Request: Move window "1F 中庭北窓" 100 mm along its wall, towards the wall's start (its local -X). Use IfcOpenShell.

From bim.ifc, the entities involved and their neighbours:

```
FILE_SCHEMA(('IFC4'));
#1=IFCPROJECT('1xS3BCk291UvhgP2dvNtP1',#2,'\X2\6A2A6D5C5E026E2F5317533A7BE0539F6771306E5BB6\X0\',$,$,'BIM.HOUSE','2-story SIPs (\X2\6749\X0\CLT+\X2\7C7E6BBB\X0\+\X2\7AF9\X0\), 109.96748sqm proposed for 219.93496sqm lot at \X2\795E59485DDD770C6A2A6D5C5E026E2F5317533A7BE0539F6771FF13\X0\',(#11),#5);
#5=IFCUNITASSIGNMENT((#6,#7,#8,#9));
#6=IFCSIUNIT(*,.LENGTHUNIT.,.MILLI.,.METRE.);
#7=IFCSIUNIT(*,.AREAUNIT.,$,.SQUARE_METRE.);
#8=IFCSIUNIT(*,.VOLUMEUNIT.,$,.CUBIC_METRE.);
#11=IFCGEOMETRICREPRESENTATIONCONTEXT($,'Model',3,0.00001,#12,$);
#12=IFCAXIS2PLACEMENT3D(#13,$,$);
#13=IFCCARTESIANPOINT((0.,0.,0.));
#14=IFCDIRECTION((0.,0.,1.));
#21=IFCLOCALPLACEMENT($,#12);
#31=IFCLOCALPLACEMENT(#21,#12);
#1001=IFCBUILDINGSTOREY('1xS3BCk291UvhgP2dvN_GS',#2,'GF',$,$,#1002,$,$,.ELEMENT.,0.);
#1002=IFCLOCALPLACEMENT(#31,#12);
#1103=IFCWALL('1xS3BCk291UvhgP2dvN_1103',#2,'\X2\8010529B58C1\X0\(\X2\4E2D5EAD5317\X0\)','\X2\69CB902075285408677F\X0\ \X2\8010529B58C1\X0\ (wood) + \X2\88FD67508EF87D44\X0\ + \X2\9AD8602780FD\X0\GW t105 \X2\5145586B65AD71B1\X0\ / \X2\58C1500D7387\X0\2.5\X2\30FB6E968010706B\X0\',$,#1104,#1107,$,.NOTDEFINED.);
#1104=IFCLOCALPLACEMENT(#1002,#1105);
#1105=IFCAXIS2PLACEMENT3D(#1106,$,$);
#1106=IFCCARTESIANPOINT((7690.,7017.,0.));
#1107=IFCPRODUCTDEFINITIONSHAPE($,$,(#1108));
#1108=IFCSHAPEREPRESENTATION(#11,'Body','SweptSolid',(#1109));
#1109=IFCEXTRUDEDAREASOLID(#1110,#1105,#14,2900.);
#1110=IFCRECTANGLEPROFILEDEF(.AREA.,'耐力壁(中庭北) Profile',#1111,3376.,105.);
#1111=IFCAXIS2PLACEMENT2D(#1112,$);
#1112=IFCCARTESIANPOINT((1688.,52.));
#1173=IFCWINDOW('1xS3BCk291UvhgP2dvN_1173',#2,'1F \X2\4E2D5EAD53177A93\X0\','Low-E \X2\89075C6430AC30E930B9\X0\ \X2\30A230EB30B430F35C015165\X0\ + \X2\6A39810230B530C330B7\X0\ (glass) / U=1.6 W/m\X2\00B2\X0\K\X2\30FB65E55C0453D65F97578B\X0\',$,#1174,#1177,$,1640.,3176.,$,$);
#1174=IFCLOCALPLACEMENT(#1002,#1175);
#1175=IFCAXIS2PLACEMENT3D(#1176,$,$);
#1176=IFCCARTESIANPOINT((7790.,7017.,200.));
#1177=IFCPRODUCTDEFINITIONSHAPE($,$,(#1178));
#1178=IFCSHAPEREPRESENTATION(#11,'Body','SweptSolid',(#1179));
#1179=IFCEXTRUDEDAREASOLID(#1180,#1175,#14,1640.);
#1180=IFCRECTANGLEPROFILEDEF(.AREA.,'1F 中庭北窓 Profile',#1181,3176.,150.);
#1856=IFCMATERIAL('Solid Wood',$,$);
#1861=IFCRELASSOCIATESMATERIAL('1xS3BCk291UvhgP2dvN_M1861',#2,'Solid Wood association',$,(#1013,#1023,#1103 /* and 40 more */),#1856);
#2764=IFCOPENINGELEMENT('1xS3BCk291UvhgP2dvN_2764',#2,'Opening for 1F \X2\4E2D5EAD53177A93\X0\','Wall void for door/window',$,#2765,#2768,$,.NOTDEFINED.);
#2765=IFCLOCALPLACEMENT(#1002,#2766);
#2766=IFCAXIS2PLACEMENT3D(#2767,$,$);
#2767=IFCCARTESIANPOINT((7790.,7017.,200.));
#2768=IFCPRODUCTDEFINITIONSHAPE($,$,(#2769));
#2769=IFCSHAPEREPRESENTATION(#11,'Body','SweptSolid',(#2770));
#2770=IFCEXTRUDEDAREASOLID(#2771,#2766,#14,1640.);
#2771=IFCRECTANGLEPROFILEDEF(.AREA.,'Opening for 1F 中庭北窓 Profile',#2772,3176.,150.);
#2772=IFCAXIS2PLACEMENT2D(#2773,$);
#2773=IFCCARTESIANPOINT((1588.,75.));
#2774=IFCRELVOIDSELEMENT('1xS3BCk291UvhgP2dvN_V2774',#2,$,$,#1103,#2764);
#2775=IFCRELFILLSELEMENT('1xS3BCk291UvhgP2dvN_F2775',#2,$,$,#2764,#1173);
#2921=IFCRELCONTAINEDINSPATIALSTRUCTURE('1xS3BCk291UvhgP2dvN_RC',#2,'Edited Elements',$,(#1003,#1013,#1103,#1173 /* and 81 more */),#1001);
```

```python
import ifcopenshell
import ifcopenshell.api.geometry
import ifcopenshell.util.placement

model = ifcopenshell.open("bim.ifc")

window = model.by_guid("1xS3BCk291UvhgP2dvN_1173")
opening = window.FillsVoids[0].RelatingOpeningElement
wall = opening.VoidsElements[0].RelatingBuildingElement

wall_matrix = ifcopenshell.util.placement.get_local_placement(wall.ObjectPlacement)
shift = wall_matrix[:3, 0] * -100.0
before = ifcopenshell.util.placement.get_local_placement(window.ObjectPlacement)[:3, 3].copy()

# The window is not placed relative to its opening, so move both.
for product in (opening, window):
    matrix = ifcopenshell.util.placement.get_local_placement(product.ObjectPlacement)
    matrix[:3, 3] += shift
    ifcopenshell.api.geometry.edit_object_placement(model, product=product, matrix=matrix, is_si=False)

after = ifcopenshell.util.placement.get_local_placement(window.ObjectPlacement)[:3, 3]
print("window moved by", (after - before).round(3) + 0.0)

model.write("bim_edited.ifc")
```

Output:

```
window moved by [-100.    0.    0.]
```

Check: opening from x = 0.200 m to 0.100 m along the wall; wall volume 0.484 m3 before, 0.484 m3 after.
